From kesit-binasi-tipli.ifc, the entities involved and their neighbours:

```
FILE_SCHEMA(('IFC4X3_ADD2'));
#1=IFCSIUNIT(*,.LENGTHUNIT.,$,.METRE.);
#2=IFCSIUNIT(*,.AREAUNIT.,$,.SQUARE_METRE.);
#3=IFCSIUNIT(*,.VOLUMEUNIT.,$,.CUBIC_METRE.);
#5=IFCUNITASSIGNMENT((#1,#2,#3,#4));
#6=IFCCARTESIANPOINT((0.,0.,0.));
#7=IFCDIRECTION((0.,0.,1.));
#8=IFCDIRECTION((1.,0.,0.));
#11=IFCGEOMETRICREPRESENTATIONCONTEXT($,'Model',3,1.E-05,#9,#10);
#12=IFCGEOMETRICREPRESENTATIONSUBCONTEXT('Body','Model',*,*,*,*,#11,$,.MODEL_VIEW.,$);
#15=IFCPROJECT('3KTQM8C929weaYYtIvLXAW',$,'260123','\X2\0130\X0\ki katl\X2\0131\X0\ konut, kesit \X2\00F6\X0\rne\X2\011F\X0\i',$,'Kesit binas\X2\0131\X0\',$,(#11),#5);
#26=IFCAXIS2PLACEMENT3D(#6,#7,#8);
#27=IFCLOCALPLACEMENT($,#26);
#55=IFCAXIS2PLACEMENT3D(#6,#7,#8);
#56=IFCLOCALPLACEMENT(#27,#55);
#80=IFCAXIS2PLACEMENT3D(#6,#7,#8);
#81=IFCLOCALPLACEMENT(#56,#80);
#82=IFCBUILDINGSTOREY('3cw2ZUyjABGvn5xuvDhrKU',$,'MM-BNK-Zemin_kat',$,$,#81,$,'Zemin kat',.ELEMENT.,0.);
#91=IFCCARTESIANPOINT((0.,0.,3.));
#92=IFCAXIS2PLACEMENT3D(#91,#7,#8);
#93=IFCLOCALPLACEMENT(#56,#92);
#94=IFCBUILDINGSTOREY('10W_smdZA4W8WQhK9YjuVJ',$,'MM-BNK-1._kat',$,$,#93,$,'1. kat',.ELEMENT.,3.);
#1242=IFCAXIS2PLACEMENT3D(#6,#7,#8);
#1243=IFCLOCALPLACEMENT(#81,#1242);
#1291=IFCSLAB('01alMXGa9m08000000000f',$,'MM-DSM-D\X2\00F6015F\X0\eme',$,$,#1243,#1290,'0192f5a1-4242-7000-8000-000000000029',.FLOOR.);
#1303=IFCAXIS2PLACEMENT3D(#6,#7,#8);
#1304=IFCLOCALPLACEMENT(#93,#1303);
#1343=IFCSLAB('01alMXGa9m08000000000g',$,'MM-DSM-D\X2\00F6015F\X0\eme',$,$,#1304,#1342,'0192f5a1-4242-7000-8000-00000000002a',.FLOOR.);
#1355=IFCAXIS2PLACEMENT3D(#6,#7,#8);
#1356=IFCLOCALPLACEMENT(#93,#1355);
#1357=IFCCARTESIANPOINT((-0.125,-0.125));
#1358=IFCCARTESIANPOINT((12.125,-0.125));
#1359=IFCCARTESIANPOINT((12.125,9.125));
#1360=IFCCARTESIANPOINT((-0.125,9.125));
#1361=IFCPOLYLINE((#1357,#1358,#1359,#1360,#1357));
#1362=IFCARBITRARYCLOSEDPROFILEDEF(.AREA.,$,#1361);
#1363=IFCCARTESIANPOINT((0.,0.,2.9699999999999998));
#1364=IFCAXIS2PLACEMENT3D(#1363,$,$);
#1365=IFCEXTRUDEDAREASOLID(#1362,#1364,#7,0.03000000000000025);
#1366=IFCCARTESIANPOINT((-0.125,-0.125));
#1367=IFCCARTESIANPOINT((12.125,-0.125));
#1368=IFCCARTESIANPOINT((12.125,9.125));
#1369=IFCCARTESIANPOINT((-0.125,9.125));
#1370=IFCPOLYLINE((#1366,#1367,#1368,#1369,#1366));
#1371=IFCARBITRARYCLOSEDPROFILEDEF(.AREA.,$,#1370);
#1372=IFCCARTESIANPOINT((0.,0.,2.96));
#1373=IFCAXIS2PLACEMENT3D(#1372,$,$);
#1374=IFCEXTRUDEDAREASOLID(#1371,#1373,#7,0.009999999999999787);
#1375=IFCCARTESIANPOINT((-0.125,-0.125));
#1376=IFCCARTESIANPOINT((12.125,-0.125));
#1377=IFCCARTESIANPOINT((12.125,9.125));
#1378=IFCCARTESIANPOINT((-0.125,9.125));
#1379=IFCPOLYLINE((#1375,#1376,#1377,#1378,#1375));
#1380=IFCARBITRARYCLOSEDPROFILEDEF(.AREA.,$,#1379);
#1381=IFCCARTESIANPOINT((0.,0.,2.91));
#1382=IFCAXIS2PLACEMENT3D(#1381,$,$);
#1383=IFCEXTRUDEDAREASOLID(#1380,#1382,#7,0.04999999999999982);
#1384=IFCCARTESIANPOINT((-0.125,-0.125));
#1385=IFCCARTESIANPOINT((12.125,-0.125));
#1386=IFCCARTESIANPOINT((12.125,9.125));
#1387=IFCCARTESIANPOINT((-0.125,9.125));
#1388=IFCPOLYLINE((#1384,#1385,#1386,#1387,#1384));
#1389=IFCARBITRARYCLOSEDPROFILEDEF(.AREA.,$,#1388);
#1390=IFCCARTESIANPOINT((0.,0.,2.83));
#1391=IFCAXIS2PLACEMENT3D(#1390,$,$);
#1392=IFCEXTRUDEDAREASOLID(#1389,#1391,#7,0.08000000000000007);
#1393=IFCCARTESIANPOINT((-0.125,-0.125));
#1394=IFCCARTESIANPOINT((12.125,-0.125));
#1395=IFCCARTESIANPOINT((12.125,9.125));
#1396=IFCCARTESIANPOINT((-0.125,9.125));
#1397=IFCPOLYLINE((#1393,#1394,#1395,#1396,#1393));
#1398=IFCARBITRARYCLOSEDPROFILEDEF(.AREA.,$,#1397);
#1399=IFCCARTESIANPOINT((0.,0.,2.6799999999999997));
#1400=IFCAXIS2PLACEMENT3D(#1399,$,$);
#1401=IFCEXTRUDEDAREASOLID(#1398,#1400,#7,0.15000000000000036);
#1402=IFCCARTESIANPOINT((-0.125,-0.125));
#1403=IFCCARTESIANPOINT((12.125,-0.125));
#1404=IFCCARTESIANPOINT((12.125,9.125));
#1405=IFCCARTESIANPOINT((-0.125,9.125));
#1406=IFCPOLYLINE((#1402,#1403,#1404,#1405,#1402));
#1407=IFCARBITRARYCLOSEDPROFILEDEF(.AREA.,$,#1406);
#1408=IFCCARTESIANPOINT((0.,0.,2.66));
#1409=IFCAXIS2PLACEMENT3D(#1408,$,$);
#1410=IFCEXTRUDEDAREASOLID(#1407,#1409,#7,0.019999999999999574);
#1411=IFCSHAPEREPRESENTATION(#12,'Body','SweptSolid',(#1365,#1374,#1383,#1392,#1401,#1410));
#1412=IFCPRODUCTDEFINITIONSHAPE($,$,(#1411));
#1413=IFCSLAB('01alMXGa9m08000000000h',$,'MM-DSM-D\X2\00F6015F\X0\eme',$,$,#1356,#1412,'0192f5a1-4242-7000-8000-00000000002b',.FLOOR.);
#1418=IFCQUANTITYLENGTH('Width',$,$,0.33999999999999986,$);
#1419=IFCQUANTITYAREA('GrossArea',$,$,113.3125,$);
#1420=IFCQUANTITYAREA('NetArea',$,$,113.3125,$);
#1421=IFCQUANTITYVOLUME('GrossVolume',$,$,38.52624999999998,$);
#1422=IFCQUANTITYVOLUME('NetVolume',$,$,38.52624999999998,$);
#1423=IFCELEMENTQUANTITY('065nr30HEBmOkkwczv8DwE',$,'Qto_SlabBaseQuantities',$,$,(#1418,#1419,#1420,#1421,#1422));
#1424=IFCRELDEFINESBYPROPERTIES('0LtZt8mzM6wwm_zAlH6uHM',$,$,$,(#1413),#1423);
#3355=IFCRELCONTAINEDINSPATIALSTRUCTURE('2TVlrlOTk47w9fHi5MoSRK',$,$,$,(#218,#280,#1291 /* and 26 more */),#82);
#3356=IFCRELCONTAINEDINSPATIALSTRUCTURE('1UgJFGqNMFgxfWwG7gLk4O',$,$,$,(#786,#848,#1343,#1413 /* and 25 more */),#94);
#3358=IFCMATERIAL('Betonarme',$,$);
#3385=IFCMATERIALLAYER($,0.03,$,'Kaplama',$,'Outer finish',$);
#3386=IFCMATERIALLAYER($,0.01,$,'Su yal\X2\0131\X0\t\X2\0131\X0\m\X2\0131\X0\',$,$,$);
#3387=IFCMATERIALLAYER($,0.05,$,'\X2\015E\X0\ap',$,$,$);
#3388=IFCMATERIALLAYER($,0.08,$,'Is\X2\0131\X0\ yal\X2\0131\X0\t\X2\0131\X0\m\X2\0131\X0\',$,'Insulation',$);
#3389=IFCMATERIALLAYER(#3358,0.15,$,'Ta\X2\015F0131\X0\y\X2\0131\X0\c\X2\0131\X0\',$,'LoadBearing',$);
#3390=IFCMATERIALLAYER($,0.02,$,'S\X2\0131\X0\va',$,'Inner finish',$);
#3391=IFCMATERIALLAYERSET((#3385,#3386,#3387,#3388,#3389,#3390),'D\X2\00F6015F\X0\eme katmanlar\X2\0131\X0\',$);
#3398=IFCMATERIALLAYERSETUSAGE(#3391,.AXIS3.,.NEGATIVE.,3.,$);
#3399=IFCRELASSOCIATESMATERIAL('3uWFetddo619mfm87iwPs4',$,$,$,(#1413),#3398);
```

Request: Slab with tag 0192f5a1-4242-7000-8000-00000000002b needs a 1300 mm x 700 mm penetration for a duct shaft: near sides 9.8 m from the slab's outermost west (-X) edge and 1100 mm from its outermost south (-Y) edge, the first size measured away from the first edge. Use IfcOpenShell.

```python
import numpy as np
import ifcopenshell
import ifcopenshell.api.feature
import ifcopenshell.api.geometry
import ifcopenshell.api.pset
import ifcopenshell.api.root
import ifcopenshell.geom
import ifcopenshell.util.element
import ifcopenshell.util.placement
import ifcopenshell.util.representation
import ifcopenshell.util.shape
import ifcopenshell.util.unit

model = ifcopenshell.open("kesit-binasi-tipli.ifc")
unit_scale = ifcopenshell.util.unit.calculate_unit_scale(model)
area_scale = ifcopenshell.util.unit.calculate_unit_scale(model, "AREAUNIT")
volume_scale = ifcopenshell.util.unit.calculate_unit_scale(model, "VOLUMEUNIT")
settings = ifcopenshell.geom.settings()


def volume(element):
    """Net volume in cubic metres, openings subtracted."""
    shape = ifcopenshell.geom.create_shape(settings, element)
    return ifcopenshell.util.shape.get_volume(shape.geometry)


slab = model.by_id(1413)
before = volume(slab)

# Extent in the slab's own axes, in metres. The edges named are its -X and -Y sides.
slab_shape = ifcopenshell.geom.create_shape(settings, slab)
vertices = ifcopenshell.util.shape.get_vertices(slab_shape.geometry)
x_min, y_min, bottom = vertices.min(axis=0)
top = vertices[:, 2].max()

opening = ifcopenshell.api.root.create_entity(model, ifc_class="IfcOpeningElement", name="Duct shaft opening", predefined_type="OPENING")
context = ifcopenshell.util.representation.get_context(model, "Model", "Body", "MODEL_VIEW")
width, depth = 1.3, 0.7
outline = [(0.0, 0.0), (width, 0.0), (width, depth), (0.0, depth), (0.0, 0.0)]
# Overshoot both faces by 50 mm so the cut is clean.
shape = ifcopenshell.api.geometry.add_slab_representation(
    model, context=context, depth=top - bottom + 0.1, polyline=outline
)
ifcopenshell.api.geometry.assign_representation(model, product=opening, representation=shape)

matrix = ifcopenshell.util.placement.get_local_placement(slab.ObjectPlacement)
matrix[:, 3] = matrix @ np.append(np.array([x_min + 9.8, y_min + 1.1, bottom - 0.05]) / unit_scale, 1.0)
ifcopenshell.api.geometry.edit_object_placement(model, product=opening, matrix=matrix, is_si=False)
ifcopenshell.api.feature.add_feature(model, feature=opening, element=slab)

after = volume(slab)

# Update the slab's stored quantities.
qto = model.by_id(ifcopenshell.util.element.get_pset(slab, "Qto_SlabBaseQuantities", should_inherit=False)["id"])
ifcopenshell.api.pset.edit_qto(model, qto=qto, properties={
    "NetArea": after / (top - bottom) / area_scale,
    "NetVolume": after / volume_scale,
})

print(f"slab volume {before:.3f} -> {after:.3f} m3")

model.write("kesit-binasi-tipli-out.ifc")
```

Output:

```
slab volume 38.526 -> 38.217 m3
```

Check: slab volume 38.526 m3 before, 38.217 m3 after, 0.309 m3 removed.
